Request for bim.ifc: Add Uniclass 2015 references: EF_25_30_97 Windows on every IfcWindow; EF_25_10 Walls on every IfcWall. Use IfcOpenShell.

First a look at what the model holds.

```python
import ifcopenshell

model = ifcopenshell.open("bim.ifc")
print(model.schema)
print("classifications:", [c.Name for c in model.by_type("IfcClassification")])
for ifc_class in ("IfcDoor", "IfcRoof", "IfcStair", "IfcWall", "IfcWindow"):
    print(ifc_class, len(model.by_type(ifc_class)))
```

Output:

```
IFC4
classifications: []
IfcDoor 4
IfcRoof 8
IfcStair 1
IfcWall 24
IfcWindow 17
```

```python
import ifcopenshell
import ifcopenshell.api.classification

model = ifcopenshell.open("bim.ifc")

system = ifcopenshell.api.classification.add_classification(model, classification="Uniclass 2015")

codes = {
    "IfcWindow": ("EF_25_30_97", "Windows"),
    "IfcWall": ("EF_25_10", "Walls"),
}
for ifc_class, (code, name) in codes.items():
    products = model.by_type(ifc_class)
    ifcopenshell.api.classification.add_reference(
        model, products=products, classification=system, identification=code, name=name
    )
    print(code, len(products))

model.write("bim-out.ifc")
```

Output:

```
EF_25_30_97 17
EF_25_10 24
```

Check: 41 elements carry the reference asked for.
